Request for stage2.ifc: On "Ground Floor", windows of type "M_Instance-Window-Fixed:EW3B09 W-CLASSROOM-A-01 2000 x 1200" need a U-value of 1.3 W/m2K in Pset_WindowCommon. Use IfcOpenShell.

First a look at what the model holds.

```python
import ifcopenshell
import ifcopenshell.util.element

model = ifcopenshell.open("stage2.ifc")
print(model.schema)
storey = next(s for s in model.by_type("IfcBuildingStorey") if s.Name == "Ground Floor")
windows = [e for e in ifcopenshell.util.element.get_decomposition(storey) if e.is_a("IfcWindow")]
seen = {}
for e in windows:
    element_type = ifcopenshell.util.element.get_type(e)
    key = (element_type.Name if element_type != e and element_type else None, ifcopenshell.util.element.get_pset(e, "Pset_WindowCommon", "ThermalTransmittance"))
    seen[key] = seen.get(key, 0) + 1
for (name, value), count in sorted(seen.items(), key=str):
    print(count, "x", name, "|", value)
```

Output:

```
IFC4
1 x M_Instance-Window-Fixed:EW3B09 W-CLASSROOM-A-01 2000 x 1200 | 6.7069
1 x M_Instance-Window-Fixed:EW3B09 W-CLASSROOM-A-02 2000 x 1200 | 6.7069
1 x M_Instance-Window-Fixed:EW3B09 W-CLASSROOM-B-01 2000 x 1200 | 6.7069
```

```python
import ifcopenshell
import ifcopenshell.api.pset
import ifcopenshell.util.element

model = ifcopenshell.open("stage2.ifc")

storey = next(s for s in model.by_type("IfcBuildingStorey") if s.Name == "Ground Floor")
windows = [e for e in ifcopenshell.util.element.get_decomposition(storey) if e.is_a("IfcWindow")]

count = 0
for e in windows:
    element_type = ifcopenshell.util.element.get_type(e)
    if element_type in (None, e) or element_type.Name != "M_Instance-Window-Fixed:EW3B09 W-CLASSROOM-A-01 2000 x 1200":
        continue
    # add_pset returns the element's existing set when there is one.
    pset = ifcopenshell.api.pset.add_pset(model, product=e, name="Pset_WindowCommon")
    ifcopenshell.api.pset.edit_pset(model, pset=pset, properties={"ThermalTransmittance": 1.3})
    count += 1

print(count, "windows updated")

model.write("stage2-out.ifc")
```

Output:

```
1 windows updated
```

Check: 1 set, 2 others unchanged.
